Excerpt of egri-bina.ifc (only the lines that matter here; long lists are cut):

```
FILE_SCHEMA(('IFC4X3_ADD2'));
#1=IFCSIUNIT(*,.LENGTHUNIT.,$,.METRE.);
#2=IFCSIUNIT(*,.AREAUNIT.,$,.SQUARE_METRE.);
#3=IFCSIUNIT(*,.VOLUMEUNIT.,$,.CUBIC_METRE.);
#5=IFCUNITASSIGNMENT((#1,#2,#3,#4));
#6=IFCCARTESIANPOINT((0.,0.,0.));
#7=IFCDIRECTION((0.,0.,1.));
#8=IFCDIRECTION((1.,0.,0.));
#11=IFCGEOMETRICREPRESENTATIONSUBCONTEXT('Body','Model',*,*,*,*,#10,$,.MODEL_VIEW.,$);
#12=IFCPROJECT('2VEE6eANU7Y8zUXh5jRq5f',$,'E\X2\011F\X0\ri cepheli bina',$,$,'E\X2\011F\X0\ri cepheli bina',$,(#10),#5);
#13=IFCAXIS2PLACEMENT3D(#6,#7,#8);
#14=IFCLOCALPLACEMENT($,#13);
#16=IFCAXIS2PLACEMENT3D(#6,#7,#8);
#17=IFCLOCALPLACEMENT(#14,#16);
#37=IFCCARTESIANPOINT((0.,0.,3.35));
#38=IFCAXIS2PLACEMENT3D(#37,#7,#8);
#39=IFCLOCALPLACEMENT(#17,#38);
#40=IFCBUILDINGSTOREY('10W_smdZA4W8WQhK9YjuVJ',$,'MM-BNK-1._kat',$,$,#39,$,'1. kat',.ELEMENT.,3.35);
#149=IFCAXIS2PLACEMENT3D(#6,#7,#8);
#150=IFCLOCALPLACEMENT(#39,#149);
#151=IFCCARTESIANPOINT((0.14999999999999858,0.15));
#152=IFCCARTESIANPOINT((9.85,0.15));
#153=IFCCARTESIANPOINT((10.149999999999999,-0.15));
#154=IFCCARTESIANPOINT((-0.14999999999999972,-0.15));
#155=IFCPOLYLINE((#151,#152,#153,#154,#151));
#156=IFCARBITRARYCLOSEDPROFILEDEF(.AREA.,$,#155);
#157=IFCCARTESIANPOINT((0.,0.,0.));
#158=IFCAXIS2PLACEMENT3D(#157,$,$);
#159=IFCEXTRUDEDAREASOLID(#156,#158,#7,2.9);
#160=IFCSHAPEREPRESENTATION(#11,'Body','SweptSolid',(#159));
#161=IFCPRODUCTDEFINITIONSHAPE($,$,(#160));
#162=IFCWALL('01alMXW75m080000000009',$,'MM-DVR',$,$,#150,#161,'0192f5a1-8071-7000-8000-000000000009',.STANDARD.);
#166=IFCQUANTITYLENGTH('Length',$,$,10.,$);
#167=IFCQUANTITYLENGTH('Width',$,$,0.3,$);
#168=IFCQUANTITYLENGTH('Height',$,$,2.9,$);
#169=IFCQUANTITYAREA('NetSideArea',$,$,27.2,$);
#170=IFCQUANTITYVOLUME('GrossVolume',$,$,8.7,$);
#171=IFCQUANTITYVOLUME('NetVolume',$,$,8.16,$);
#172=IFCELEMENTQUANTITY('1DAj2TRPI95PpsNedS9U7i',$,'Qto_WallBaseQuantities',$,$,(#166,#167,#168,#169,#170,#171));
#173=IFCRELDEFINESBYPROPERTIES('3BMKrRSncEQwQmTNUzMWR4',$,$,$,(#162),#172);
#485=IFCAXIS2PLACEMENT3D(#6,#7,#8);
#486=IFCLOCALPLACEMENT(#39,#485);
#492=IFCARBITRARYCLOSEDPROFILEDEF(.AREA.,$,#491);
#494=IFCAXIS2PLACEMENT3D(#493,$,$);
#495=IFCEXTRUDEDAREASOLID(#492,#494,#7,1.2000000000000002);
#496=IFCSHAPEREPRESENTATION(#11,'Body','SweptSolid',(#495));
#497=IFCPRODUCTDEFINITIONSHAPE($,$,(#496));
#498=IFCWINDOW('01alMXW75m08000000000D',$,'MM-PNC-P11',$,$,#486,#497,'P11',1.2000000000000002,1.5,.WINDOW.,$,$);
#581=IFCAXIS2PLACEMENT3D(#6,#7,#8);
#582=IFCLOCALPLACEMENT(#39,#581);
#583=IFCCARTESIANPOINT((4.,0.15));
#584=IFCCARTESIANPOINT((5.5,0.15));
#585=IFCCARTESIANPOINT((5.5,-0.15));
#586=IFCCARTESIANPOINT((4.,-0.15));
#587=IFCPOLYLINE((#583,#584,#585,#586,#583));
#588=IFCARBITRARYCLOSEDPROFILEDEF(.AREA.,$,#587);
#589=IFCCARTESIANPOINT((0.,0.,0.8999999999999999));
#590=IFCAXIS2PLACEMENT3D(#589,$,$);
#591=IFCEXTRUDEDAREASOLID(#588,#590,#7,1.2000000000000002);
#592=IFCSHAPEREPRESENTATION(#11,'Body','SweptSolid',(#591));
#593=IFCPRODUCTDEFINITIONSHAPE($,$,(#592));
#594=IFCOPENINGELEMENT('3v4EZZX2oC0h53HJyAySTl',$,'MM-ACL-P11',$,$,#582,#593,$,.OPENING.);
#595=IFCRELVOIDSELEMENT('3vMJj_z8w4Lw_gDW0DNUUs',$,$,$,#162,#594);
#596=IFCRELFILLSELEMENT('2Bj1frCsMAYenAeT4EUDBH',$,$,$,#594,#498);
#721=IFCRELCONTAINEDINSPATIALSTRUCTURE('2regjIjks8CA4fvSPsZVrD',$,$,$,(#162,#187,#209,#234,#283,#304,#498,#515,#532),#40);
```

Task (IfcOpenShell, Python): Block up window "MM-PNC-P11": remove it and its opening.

```python
import ifcopenshell
import ifcopenshell.api.feature
import ifcopenshell.api.pset
import ifcopenshell.api.root
import ifcopenshell.geom
import ifcopenshell.util.element
import ifcopenshell.util.shape
import ifcopenshell.util.unit

model = ifcopenshell.open("egri-bina.ifc")
area_scale = ifcopenshell.util.unit.calculate_unit_scale(model, "AREAUNIT")
volume_scale = ifcopenshell.util.unit.calculate_unit_scale(model, "VOLUMEUNIT")
settings = ifcopenshell.geom.settings()


def volume(element):
    """Net volume in cubic metres, openings subtracted."""
    shape = ifcopenshell.geom.create_shape(settings, element)
    return ifcopenshell.util.shape.get_volume(shape.geometry)


window = model.by_id(498)
opening = window.FillsVoids[0].RelatingOpeningElement
wall = opening.VoidsElements[0].RelatingBuildingElement
before = volume(wall)

ifcopenshell.api.root.remove_product(model, product=window)
ifcopenshell.api.feature.remove_feature(model, feature=opening)

after = volume(wall)
thickness = 0.3  # wall thickness in metres

# Update the wall's stored quantities.
qto = model.by_id(ifcopenshell.util.element.get_pset(wall, "Qto_WallBaseQuantities", should_inherit=False)["id"])
ifcopenshell.api.pset.edit_qto(model, qto=qto, properties={
    "NetSideArea": after / thickness / area_scale,
    "NetVolume": after / volume_scale,
})

print(f"wall volume {before:.3f} -> {after:.3f} m3")

model.write("egri-bina_rev.ifc")
```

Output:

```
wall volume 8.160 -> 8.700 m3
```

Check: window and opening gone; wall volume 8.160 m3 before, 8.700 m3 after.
